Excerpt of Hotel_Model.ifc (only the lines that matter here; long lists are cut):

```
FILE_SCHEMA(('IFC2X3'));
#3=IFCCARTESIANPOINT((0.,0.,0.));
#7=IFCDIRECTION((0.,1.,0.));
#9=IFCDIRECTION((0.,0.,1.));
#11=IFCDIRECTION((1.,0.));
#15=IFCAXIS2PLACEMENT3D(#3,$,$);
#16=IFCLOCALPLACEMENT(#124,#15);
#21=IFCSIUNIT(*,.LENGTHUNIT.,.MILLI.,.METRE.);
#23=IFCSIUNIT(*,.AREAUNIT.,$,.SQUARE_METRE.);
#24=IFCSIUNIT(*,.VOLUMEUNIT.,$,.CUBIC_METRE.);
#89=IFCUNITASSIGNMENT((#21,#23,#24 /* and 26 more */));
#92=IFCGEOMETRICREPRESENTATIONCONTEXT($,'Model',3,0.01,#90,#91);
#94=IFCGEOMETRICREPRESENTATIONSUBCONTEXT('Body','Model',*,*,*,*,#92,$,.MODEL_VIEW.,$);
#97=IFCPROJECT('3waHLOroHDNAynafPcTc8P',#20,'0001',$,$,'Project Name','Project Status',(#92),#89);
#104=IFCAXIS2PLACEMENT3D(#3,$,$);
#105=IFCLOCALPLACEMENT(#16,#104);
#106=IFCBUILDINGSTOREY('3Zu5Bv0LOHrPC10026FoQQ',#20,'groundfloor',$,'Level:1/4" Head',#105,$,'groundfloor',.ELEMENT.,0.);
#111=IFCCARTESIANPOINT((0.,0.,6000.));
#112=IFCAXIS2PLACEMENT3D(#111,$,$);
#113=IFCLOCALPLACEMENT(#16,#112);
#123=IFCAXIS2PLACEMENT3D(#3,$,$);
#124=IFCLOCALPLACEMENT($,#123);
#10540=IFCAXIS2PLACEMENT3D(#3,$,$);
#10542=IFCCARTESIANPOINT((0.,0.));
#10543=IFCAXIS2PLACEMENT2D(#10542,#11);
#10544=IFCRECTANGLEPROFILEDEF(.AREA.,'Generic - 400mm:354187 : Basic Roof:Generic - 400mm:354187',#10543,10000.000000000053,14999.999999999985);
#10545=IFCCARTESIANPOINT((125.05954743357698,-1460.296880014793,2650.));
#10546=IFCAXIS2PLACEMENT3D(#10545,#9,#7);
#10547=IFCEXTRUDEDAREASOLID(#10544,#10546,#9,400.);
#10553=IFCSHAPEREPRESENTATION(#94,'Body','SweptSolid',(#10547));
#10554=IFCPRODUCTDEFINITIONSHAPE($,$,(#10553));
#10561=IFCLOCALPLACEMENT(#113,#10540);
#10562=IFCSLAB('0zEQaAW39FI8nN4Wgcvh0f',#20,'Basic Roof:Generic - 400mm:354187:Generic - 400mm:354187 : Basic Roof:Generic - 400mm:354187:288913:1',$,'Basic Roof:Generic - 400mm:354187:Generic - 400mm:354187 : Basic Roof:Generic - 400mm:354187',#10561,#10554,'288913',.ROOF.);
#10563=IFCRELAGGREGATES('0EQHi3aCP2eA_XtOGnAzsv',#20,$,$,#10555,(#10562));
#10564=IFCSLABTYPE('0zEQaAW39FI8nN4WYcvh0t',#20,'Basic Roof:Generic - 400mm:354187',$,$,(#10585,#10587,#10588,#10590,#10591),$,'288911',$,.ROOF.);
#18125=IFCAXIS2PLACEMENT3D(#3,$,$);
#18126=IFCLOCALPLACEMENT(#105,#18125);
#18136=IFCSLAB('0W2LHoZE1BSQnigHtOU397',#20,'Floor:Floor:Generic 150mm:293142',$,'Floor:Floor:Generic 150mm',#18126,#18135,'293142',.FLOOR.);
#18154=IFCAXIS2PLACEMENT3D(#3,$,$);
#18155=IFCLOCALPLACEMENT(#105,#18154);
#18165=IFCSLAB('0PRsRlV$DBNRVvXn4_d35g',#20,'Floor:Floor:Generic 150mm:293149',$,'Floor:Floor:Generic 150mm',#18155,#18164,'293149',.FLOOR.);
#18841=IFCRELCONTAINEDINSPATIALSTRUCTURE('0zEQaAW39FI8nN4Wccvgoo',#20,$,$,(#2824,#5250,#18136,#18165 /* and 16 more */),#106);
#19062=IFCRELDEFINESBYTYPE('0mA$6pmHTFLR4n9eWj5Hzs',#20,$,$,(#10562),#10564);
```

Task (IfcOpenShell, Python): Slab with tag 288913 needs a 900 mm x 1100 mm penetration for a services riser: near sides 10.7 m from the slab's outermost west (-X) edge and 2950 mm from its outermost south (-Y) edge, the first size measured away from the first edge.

```python
import numpy as np
import ifcopenshell
import ifcopenshell.api.feature
import ifcopenshell.api.geometry
import ifcopenshell.api.root
import ifcopenshell.geom
import ifcopenshell.util.placement
import ifcopenshell.util.representation
import ifcopenshell.util.shape
import ifcopenshell.util.unit

model = ifcopenshell.open("Hotel_Model.ifc")
unit_scale = ifcopenshell.util.unit.calculate_unit_scale(model)
settings = ifcopenshell.geom.settings()


def volume(element):
    """Net volume in cubic metres, openings subtracted."""
    shape = ifcopenshell.geom.create_shape(settings, element)
    return ifcopenshell.util.shape.get_volume(shape.geometry)


slab = model.by_guid("0zEQaAW39FI8nN4Wgcvh0f")
before = volume(slab)

# Extent in the slab's own axes, in metres. The edges named are its -X and -Y sides.
slab_shape = ifcopenshell.geom.create_shape(settings, slab)
vertices = ifcopenshell.util.shape.get_vertices(slab_shape.geometry)
x_min, y_min, bottom = vertices.min(axis=0)
top = vertices[:, 2].max()

opening = ifcopenshell.api.root.create_entity(model, ifc_class="IfcOpeningElement", name="Services riser opening")
context = ifcopenshell.util.representation.get_context(model, "Model", "Body", "MODEL_VIEW")
width, depth = 0.9, 1.1
outline = [(0.0, 0.0), (width, 0.0), (width, depth), (0.0, depth), (0.0, 0.0)]
# Overshoot both faces by 50 mm so the cut is clean.
shape = ifcopenshell.api.geometry.add_slab_representation(
    model, context=context, depth=top - bottom + 0.1, polyline=outline
)
ifcopenshell.api.geometry.assign_representation(model, product=opening, representation=shape)

matrix = ifcopenshell.util.placement.get_local_placement(slab.ObjectPlacement)
matrix[:, 3] = matrix @ np.append(np.array([x_min + 10.7, y_min + 2.95, bottom - 0.05]) / unit_scale, 1.0)
ifcopenshell.api.geometry.edit_object_placement(model, product=opening, matrix=matrix, is_si=False)
ifcopenshell.api.feature.add_feature(model, feature=opening, element=slab)

after = volume(slab)

print(f"slab volume {before:.3f} -> {after:.3f} m3")

model.write("Hotel_Model-out.ifc")
```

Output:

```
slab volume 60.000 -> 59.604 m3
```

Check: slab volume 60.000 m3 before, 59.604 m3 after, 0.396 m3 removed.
